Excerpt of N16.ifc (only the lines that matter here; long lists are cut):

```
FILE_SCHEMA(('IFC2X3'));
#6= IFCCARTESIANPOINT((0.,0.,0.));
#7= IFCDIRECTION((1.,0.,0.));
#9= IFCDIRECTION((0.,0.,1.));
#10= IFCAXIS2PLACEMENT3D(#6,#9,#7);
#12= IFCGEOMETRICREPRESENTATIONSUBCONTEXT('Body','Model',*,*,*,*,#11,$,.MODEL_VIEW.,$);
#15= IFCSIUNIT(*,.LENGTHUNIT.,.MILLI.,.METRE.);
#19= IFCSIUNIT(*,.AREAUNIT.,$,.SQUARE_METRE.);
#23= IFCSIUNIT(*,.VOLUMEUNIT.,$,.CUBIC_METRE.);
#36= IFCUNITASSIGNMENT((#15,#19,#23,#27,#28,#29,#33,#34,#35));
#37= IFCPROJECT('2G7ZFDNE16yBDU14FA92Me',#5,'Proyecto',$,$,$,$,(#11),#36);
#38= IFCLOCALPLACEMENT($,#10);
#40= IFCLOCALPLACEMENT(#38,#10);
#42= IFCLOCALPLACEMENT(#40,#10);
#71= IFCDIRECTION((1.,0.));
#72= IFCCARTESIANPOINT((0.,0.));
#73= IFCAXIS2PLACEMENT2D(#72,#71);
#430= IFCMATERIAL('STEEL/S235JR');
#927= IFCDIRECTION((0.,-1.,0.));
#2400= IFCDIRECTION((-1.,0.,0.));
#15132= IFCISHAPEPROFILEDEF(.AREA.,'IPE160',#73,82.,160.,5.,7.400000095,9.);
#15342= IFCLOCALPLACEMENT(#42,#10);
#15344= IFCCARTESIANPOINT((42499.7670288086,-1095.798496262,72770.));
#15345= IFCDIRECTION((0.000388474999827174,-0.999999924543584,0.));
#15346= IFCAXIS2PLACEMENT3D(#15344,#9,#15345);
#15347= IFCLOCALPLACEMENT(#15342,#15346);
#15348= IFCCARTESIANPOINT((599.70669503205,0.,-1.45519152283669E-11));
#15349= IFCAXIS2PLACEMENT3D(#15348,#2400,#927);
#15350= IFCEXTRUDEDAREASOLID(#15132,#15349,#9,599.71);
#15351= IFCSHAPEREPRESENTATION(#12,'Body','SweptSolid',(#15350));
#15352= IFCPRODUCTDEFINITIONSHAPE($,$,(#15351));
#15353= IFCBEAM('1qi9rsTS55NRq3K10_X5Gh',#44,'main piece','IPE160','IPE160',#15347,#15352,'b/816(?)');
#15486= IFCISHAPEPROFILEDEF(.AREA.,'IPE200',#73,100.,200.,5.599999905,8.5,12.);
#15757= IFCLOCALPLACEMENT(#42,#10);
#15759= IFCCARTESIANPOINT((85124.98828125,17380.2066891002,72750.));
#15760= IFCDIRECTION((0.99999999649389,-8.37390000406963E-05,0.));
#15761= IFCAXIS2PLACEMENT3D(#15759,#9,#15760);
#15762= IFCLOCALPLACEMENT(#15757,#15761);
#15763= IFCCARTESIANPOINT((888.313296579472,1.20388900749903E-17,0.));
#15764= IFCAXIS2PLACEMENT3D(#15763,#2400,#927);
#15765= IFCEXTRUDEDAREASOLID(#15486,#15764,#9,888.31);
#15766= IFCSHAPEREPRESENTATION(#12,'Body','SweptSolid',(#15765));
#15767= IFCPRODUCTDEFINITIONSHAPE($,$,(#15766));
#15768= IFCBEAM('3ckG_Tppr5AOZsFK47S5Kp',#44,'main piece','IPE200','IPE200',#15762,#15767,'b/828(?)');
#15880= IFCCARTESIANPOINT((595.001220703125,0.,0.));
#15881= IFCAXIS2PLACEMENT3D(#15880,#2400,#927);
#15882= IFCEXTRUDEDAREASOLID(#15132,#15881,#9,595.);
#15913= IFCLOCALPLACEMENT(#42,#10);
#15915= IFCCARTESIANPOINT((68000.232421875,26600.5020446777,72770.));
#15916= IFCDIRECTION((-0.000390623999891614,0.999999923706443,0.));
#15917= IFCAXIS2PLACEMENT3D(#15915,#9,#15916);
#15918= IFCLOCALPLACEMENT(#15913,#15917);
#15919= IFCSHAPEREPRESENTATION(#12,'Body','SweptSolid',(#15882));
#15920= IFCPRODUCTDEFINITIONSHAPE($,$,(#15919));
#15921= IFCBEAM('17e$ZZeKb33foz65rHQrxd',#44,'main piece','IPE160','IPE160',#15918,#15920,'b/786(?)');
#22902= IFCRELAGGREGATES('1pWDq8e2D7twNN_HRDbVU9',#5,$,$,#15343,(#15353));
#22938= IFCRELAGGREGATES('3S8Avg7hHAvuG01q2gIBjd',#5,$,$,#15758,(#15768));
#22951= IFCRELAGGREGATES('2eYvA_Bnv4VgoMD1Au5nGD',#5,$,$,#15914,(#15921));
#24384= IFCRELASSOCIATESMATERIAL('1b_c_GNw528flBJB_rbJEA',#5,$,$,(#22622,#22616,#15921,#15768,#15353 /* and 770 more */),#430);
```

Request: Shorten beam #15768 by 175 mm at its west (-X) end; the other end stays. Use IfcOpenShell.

```python
import ifcopenshell
import ifcopenshell.util.representation

model = ifcopenshell.open("N16.ifc")

member = model.by_guid("3ckG_Tppr5AOZsFK47S5Kp")
change = -175.0

# The extrusion runs towards the end named, so only its depth changes.
body = ifcopenshell.util.representation.get_representation(member, "Model", "Body")
solid = body.Items[0]
old_length = solid.Depth
solid.Depth += change

print(f"length {old_length:g} -> {solid.Depth:g}")

model.write("N16_rev.ifc")
```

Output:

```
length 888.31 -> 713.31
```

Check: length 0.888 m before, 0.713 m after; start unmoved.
